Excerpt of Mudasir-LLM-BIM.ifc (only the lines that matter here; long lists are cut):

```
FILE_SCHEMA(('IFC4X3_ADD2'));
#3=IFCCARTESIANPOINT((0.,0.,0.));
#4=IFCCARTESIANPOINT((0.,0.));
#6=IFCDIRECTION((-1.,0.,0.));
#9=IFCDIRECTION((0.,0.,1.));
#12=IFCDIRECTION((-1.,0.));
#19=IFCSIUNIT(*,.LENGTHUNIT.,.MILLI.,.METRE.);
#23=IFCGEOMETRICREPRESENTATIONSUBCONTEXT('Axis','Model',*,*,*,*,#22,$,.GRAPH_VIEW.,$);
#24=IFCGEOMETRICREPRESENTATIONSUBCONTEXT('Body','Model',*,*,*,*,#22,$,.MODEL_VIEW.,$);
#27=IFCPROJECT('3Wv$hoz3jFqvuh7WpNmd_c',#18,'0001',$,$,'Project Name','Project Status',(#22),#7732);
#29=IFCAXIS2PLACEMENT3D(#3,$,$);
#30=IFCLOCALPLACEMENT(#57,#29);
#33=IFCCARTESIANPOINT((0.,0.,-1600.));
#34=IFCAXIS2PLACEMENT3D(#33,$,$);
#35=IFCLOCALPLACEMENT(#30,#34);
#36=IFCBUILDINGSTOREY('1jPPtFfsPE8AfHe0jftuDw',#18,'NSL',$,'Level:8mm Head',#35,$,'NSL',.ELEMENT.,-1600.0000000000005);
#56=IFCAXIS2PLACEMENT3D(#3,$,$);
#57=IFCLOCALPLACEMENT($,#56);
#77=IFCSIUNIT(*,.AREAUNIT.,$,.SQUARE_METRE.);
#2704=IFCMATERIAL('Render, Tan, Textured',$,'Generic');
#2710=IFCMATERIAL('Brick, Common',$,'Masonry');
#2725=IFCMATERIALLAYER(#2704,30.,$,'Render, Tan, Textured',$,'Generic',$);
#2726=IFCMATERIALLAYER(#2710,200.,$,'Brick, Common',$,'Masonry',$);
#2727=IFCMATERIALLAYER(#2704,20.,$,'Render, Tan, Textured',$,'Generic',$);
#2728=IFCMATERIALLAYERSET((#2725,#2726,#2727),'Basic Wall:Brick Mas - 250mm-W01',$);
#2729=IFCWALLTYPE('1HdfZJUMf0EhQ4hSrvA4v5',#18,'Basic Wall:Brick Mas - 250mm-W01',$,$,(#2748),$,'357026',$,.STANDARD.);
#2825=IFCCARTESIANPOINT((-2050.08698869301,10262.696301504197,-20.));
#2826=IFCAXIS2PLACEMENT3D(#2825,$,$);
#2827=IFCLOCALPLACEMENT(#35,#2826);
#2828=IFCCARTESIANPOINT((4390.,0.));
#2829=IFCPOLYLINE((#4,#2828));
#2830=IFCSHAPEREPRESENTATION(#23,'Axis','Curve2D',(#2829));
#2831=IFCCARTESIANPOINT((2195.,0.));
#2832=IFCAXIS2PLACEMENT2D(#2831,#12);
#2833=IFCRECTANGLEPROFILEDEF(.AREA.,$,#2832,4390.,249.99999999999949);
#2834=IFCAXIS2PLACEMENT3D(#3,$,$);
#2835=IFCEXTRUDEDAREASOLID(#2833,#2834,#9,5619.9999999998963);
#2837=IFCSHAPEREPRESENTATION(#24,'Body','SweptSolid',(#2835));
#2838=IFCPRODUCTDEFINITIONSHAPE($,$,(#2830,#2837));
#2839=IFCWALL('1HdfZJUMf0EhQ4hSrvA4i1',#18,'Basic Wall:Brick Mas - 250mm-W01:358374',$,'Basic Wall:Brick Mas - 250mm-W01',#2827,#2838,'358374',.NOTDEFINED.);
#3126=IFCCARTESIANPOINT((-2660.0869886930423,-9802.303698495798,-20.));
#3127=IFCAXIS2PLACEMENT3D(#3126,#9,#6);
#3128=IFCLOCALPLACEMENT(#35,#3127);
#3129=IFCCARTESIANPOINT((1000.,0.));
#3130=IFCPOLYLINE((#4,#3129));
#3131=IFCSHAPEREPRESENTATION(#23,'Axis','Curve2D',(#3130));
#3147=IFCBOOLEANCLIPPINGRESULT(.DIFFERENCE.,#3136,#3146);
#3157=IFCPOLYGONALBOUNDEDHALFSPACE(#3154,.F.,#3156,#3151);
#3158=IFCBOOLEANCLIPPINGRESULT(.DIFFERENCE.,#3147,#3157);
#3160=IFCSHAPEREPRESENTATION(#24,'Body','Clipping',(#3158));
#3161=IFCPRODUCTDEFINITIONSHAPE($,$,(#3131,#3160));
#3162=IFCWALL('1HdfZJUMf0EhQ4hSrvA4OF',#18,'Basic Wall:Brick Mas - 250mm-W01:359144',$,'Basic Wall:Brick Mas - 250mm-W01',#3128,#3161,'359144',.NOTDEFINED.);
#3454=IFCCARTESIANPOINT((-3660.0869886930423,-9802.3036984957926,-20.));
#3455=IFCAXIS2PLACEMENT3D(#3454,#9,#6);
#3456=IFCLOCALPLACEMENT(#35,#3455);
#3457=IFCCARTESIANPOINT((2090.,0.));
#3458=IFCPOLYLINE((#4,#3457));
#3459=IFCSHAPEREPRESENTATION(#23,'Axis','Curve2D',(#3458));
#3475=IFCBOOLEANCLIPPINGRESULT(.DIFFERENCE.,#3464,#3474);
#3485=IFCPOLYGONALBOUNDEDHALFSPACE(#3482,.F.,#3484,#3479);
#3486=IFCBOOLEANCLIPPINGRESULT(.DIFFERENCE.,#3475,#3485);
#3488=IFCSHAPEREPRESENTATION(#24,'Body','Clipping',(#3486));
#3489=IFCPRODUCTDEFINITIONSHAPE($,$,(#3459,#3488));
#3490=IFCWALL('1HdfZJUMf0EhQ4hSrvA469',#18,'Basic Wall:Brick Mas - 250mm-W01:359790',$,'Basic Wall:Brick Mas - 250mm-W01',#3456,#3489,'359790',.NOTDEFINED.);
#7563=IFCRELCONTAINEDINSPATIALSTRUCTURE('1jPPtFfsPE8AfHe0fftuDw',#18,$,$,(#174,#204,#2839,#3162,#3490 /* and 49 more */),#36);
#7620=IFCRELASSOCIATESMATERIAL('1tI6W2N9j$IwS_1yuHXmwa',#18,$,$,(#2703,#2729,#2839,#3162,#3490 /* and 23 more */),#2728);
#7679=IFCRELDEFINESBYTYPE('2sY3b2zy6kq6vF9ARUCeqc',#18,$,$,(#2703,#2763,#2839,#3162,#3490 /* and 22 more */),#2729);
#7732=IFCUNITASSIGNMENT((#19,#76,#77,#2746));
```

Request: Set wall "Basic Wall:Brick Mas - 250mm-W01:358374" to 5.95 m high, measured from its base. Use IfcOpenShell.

```python
import ifcopenshell
import ifcopenshell.geom
import ifcopenshell.util.representation
import ifcopenshell.util.shape
import ifcopenshell.util.unit

model = ifcopenshell.open("Mudasir-LLM-BIM.ifc")
unit_scale = ifcopenshell.util.unit.calculate_unit_scale(model)
settings = ifcopenshell.geom.settings()


def volume(element):
    """Net volume in cubic metres, openings subtracted."""
    shape = ifcopenshell.geom.create_shape(settings, element)
    return ifcopenshell.util.shape.get_volume(shape.geometry)


wall = model.by_id(2839)
before = volume(wall)

body = ifcopenshell.util.representation.get_representation(wall, "Model", "Body")
solid = body.Items[0]
old_height = solid.Depth
solid.Depth = 5.95 / unit_scale
after = volume(wall)

print(f"height {old_height:g} -> {solid.Depth:g}, volume {before:.3f} -> {after:.3f} m3")

model.write("Mudasir-LLM-BIM_updated.ifc")
```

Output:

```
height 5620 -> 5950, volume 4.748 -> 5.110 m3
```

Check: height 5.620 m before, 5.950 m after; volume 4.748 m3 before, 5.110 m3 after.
